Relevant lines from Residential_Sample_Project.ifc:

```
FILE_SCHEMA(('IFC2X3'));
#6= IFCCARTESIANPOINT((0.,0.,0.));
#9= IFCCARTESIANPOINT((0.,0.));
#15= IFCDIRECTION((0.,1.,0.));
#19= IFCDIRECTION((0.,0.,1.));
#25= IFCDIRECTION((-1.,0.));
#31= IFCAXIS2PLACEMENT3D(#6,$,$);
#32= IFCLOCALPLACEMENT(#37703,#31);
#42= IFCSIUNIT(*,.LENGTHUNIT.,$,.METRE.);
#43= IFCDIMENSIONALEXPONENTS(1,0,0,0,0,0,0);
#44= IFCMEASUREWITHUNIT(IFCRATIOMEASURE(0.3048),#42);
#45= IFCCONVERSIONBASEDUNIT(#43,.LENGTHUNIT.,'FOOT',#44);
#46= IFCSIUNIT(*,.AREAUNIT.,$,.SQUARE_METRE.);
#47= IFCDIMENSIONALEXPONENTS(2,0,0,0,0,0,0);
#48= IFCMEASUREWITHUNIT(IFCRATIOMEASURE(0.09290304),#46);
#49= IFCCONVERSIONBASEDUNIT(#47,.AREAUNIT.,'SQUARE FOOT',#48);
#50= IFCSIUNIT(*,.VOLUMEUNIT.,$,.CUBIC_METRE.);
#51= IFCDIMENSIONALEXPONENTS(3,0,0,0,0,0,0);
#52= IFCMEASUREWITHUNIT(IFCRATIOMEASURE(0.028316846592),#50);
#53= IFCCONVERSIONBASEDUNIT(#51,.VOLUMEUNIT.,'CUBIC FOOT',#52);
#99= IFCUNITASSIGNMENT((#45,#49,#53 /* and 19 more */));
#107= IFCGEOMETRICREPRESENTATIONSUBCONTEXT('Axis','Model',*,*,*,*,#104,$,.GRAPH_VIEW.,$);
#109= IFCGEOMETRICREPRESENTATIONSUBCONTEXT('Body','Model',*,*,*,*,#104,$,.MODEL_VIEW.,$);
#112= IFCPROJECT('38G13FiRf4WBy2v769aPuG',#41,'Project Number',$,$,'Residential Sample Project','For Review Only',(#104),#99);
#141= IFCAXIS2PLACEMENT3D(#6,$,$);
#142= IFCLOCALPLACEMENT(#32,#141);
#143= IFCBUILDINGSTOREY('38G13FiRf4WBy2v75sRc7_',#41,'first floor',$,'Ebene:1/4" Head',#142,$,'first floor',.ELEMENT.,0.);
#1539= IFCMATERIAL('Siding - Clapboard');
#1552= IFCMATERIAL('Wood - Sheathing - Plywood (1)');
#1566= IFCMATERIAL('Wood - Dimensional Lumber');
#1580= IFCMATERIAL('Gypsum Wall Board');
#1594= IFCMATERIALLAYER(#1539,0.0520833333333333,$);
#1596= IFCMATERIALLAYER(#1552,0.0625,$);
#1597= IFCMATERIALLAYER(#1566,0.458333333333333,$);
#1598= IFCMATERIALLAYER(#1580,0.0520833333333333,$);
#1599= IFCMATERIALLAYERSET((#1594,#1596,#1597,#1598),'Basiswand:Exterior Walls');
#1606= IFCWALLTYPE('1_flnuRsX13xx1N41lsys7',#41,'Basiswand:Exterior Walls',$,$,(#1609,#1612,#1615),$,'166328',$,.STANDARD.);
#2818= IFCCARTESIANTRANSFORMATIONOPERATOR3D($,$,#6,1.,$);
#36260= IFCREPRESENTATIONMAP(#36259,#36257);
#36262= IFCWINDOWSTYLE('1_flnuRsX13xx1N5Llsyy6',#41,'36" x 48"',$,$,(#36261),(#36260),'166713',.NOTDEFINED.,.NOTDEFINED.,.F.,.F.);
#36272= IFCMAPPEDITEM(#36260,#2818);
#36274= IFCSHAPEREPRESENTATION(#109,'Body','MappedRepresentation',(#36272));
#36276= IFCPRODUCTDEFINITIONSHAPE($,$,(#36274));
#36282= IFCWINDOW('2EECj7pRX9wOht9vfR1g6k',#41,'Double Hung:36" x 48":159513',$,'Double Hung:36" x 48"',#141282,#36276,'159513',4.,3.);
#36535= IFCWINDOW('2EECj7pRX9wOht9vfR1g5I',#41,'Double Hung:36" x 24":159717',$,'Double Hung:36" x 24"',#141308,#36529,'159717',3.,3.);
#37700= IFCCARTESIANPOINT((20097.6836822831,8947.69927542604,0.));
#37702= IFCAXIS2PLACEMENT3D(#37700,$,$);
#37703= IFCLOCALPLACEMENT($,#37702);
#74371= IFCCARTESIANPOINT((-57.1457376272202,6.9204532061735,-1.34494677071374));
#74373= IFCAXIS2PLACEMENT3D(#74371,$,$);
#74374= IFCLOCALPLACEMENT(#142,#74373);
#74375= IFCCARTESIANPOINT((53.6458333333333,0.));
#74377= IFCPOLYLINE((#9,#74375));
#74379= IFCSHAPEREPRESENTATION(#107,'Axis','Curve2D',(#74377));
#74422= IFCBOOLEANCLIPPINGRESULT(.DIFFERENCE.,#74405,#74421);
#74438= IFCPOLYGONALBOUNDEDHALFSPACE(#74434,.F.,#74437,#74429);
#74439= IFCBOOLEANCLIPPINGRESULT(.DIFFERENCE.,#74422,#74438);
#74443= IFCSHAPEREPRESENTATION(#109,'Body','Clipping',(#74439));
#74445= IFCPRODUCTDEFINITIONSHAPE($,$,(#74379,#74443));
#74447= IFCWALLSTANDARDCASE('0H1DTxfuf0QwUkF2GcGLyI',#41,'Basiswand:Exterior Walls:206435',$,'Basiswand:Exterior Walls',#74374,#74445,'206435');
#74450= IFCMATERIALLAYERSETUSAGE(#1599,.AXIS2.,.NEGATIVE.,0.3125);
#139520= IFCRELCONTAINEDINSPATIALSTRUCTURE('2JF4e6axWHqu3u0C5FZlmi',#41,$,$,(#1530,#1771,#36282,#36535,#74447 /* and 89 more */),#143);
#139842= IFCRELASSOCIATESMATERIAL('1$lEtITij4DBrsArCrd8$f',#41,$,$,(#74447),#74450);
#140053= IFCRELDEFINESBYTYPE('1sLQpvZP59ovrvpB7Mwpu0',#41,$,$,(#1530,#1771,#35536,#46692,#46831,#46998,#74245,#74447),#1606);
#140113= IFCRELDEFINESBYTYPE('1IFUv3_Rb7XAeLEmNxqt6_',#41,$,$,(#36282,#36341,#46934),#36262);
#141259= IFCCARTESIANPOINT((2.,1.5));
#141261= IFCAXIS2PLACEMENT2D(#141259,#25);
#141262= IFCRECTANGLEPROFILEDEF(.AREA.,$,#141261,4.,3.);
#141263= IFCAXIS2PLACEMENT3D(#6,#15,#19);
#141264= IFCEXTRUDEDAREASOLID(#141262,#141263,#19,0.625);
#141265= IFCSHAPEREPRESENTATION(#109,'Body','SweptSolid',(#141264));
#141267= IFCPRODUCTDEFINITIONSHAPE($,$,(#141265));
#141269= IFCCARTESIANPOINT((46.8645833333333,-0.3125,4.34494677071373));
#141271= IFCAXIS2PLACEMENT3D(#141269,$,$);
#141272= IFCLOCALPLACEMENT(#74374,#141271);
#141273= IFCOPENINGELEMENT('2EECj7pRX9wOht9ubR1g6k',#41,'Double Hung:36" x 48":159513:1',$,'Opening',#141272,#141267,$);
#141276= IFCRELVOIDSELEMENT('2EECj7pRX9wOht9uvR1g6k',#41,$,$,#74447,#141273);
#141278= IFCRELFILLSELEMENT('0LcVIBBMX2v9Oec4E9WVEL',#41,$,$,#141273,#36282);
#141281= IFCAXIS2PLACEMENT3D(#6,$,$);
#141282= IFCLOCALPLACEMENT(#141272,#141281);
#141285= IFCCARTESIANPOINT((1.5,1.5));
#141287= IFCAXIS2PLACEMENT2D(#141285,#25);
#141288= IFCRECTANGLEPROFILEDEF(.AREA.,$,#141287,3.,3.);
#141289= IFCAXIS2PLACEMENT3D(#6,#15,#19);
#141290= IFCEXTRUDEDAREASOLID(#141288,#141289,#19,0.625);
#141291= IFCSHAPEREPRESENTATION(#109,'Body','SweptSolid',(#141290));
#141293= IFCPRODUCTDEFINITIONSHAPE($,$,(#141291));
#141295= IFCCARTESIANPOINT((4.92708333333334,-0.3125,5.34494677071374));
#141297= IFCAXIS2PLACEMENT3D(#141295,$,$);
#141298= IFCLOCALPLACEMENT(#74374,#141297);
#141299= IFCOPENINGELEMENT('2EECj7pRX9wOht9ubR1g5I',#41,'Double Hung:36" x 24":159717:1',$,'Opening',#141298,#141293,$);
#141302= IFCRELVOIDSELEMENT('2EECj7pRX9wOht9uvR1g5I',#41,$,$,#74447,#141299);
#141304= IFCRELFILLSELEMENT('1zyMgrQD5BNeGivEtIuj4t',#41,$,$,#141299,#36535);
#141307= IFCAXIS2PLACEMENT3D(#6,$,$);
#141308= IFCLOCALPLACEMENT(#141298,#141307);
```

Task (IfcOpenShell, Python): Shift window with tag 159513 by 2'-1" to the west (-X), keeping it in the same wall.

```python
import ifcopenshell
import ifcopenshell.api.geometry
import ifcopenshell.util.placement
import ifcopenshell.util.unit

model = ifcopenshell.open("Residential_Sample_Project.ifc")
unit_scale = ifcopenshell.util.unit.calculate_unit_scale(model)

window = model.by_guid("2EECj7pRX9wOht9vfR1g6k")
opening = window.FillsVoids[0].RelatingOpeningElement
wall = opening.VoidsElements[0].RelatingBuildingElement

wall_matrix = ifcopenshell.util.placement.get_local_placement(wall.ObjectPlacement)
shift = wall_matrix[:3, 0] * -25 * 0.0254 / unit_scale
before = ifcopenshell.util.placement.get_local_placement(window.ObjectPlacement)[:3, 3].copy()

# The window is placed relative to its opening, so it follows when the opening moves.
matrix = ifcopenshell.util.placement.get_local_placement(opening.ObjectPlacement)
matrix[:3, 3] += shift
ifcopenshell.api.geometry.edit_object_placement(
    model, product=opening, matrix=matrix, is_si=False, should_transform_children=True
)

after = ifcopenshell.util.placement.get_local_placement(window.ObjectPlacement)[:3, 3]
print("window moved by", (after - before).round(3) + 0.0)

model.write("Residential_Sample_Project_edited.ifc")
```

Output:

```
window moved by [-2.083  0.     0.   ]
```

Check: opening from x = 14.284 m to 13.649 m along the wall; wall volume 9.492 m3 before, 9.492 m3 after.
